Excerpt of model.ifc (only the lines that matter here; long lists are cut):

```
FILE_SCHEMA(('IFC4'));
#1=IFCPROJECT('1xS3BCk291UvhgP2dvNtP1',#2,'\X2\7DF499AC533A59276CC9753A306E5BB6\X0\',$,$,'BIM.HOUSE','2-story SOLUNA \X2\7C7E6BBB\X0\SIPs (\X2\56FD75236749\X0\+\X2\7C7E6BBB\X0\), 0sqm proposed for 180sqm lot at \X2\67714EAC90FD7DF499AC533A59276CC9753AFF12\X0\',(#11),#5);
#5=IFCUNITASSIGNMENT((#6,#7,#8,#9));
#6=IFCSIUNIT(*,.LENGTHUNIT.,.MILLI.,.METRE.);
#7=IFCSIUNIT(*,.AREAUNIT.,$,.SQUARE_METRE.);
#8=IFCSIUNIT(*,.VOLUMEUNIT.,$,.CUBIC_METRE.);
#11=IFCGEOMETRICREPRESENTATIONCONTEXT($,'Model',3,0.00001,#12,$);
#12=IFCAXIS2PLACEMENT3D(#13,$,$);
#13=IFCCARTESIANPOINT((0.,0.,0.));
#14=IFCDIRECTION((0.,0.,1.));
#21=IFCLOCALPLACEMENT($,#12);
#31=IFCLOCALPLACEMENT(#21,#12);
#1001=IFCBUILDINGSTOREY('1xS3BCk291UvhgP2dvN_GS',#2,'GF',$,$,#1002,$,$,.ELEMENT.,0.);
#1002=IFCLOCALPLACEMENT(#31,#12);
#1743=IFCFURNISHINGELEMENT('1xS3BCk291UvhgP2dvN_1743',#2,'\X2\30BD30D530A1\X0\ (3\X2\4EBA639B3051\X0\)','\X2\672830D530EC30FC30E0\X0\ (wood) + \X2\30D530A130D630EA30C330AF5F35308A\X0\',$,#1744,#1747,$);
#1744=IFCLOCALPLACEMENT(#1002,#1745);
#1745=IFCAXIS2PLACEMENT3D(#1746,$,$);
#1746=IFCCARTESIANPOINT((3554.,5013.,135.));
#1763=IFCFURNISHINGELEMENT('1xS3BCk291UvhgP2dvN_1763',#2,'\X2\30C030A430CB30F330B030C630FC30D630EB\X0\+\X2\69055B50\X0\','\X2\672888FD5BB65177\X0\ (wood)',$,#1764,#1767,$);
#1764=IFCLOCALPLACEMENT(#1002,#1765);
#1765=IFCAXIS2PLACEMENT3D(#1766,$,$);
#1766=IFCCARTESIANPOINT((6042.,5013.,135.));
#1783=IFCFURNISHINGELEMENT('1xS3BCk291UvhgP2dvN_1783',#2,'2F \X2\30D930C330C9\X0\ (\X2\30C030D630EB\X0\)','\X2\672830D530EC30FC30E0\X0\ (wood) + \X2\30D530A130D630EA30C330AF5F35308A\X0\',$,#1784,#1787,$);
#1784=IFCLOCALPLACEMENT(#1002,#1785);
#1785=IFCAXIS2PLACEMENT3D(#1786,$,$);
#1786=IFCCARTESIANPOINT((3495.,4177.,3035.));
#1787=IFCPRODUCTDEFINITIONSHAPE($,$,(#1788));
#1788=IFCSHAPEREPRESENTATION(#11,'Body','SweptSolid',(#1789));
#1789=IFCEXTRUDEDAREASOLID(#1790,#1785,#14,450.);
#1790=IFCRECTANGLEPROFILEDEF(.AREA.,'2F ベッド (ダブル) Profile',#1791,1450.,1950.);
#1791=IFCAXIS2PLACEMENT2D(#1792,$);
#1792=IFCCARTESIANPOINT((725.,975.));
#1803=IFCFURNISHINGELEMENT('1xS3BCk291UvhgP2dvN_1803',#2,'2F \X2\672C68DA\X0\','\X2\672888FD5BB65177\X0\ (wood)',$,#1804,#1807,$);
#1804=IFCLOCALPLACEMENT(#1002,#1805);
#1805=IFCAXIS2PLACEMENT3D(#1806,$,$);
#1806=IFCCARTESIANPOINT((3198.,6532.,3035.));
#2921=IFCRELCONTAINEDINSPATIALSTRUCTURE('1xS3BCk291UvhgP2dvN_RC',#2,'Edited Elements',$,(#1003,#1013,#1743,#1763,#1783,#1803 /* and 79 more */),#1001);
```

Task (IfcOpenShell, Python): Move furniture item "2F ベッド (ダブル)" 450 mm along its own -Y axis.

```python
import ifcopenshell
import ifcopenshell.api.geometry
import ifcopenshell.util.placement

model = ifcopenshell.open("model.ifc")

item = model.by_guid("1xS3BCk291UvhgP2dvN_1783")
matrix = ifcopenshell.util.placement.get_local_placement(item.ObjectPlacement)
matrix[:3, 3] -= matrix[:3, 1] * 450.0
ifcopenshell.api.geometry.edit_object_placement(model, product=item, matrix=matrix, is_si=False)

print(ifcopenshell.util.placement.get_local_placement(item.ObjectPlacement).round(3) + 0.0)

model.write("model-out.ifc")
```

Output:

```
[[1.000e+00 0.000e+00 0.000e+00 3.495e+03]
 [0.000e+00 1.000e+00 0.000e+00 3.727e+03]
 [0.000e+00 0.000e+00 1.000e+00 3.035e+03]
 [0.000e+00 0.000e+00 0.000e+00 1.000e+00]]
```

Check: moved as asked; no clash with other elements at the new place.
